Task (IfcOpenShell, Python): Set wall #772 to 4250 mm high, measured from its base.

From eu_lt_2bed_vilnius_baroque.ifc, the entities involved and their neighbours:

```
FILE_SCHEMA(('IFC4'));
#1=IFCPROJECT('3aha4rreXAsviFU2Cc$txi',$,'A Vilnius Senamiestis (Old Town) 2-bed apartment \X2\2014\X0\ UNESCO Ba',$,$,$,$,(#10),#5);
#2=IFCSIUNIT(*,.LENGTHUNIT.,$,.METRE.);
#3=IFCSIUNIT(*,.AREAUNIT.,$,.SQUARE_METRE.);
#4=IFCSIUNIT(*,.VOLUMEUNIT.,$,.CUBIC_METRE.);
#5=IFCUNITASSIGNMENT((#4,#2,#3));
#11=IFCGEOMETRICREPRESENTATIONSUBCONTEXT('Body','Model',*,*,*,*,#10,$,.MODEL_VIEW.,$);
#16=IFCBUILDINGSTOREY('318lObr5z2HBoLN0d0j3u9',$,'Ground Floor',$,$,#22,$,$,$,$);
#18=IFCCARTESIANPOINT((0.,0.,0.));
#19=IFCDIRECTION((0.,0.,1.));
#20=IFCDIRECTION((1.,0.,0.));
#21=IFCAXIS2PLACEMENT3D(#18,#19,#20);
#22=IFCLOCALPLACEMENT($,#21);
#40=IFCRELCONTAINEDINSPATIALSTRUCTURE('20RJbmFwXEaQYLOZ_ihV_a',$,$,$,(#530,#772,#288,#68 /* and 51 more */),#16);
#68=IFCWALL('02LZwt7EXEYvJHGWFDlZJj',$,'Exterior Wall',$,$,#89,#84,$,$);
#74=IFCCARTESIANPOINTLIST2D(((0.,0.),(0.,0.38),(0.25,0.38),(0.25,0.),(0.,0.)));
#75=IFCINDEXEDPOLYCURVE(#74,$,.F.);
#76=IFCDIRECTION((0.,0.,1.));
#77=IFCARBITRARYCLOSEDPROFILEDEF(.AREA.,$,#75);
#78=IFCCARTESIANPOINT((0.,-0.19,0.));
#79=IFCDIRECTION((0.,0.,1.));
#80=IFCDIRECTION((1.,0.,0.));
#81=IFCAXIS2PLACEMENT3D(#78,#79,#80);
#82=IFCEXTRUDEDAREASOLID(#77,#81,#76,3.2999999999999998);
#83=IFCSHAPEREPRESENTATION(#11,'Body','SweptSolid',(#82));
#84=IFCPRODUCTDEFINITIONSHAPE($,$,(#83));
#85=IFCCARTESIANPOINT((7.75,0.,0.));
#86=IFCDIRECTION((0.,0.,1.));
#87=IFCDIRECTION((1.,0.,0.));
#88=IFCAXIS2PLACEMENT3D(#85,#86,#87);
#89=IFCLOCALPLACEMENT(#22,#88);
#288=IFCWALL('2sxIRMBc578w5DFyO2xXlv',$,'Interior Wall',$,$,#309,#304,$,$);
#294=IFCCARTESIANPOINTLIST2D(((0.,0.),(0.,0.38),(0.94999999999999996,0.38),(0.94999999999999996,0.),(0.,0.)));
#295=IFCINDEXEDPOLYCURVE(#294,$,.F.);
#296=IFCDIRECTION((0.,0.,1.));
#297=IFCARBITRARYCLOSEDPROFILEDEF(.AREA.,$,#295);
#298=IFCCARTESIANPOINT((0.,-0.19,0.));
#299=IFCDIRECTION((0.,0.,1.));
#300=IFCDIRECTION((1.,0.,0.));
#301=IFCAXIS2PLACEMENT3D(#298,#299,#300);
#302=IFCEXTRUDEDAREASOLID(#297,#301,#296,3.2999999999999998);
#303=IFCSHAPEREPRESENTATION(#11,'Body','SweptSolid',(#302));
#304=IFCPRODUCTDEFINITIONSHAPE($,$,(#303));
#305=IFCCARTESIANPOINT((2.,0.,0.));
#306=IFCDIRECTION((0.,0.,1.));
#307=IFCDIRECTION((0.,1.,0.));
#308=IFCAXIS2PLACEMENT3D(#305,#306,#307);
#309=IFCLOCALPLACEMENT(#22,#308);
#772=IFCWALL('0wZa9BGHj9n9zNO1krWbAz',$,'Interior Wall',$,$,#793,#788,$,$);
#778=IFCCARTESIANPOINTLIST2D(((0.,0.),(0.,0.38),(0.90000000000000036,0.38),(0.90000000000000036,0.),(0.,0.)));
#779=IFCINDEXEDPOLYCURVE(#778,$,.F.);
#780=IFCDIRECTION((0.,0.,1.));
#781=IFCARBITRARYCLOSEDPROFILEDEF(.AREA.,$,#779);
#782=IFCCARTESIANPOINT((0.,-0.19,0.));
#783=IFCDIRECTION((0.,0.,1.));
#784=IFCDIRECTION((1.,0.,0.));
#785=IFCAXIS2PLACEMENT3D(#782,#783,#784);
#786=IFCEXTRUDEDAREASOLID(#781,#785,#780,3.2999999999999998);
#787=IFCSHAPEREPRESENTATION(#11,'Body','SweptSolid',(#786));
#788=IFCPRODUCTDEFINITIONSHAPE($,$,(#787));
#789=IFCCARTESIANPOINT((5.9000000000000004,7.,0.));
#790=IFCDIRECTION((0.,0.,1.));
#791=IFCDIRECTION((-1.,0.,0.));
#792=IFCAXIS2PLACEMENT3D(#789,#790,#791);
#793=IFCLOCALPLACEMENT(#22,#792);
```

```python
import ifcopenshell
import ifcopenshell.geom
import ifcopenshell.util.representation
import ifcopenshell.util.shape

model = ifcopenshell.open("eu_lt_2bed_vilnius_baroque.ifc")
settings = ifcopenshell.geom.settings()


def volume(element):
    """Net volume in cubic metres, openings subtracted."""
    shape = ifcopenshell.geom.create_shape(settings, element)
    return ifcopenshell.util.shape.get_volume(shape.geometry)


wall = model.by_guid("0wZa9BGHj9n9zNO1krWbAz")
before = volume(wall)

body = ifcopenshell.util.representation.get_representation(wall, "Model", "Body")
solid = body.Items[0]
old_height = solid.Depth
solid.Depth = 4.25
after = volume(wall)

print(f"height {old_height:g} -> {solid.Depth:g}, volume {before:.3f} -> {after:.3f} m3")

model.write("eu_lt_2bed_vilnius_baroque_updated.ifc")
```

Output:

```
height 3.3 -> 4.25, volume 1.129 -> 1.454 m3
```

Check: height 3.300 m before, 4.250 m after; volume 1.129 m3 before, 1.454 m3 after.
